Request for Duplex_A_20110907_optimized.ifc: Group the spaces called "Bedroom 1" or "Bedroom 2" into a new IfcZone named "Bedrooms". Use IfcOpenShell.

First a look at what the model holds.

```python
import ifcopenshell

model = ifcopenshell.open("Duplex_A_20110907_optimized.ifc")
print(model.schema)
seen = {}
for space in model.by_type("IfcSpace"):
    seen[space.LongName] = seen.get(space.LongName, 0) + 1
for name, count in sorted(seen.items(), key=str):
    print(count, "x", name)
print("zones:", [z.Name for z in model.by_type("IfcZone")][:20])
```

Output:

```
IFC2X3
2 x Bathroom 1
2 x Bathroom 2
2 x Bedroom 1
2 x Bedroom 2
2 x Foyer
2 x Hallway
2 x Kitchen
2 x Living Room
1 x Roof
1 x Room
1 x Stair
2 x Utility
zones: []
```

```python
import ifcopenshell
import ifcopenshell.api.group
import ifcopenshell.api.root

model = ifcopenshell.open("Duplex_A_20110907_optimized.ifc")

names = {"Bedroom 1", "Bedroom 2"}
spaces = [s for s in model.by_type("IfcSpace") if s.LongName in names]

zone = ifcopenshell.api.root.create_entity(model, ifc_class="IfcZone", name="Bedrooms")
ifcopenshell.api.group.assign_group(model, products=spaces, group=zone)
print(len(spaces), "spaces in", zone.Name)

model.write("Duplex_A_20110907_optimized_v2.ifc")
```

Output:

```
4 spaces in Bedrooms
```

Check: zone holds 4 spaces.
